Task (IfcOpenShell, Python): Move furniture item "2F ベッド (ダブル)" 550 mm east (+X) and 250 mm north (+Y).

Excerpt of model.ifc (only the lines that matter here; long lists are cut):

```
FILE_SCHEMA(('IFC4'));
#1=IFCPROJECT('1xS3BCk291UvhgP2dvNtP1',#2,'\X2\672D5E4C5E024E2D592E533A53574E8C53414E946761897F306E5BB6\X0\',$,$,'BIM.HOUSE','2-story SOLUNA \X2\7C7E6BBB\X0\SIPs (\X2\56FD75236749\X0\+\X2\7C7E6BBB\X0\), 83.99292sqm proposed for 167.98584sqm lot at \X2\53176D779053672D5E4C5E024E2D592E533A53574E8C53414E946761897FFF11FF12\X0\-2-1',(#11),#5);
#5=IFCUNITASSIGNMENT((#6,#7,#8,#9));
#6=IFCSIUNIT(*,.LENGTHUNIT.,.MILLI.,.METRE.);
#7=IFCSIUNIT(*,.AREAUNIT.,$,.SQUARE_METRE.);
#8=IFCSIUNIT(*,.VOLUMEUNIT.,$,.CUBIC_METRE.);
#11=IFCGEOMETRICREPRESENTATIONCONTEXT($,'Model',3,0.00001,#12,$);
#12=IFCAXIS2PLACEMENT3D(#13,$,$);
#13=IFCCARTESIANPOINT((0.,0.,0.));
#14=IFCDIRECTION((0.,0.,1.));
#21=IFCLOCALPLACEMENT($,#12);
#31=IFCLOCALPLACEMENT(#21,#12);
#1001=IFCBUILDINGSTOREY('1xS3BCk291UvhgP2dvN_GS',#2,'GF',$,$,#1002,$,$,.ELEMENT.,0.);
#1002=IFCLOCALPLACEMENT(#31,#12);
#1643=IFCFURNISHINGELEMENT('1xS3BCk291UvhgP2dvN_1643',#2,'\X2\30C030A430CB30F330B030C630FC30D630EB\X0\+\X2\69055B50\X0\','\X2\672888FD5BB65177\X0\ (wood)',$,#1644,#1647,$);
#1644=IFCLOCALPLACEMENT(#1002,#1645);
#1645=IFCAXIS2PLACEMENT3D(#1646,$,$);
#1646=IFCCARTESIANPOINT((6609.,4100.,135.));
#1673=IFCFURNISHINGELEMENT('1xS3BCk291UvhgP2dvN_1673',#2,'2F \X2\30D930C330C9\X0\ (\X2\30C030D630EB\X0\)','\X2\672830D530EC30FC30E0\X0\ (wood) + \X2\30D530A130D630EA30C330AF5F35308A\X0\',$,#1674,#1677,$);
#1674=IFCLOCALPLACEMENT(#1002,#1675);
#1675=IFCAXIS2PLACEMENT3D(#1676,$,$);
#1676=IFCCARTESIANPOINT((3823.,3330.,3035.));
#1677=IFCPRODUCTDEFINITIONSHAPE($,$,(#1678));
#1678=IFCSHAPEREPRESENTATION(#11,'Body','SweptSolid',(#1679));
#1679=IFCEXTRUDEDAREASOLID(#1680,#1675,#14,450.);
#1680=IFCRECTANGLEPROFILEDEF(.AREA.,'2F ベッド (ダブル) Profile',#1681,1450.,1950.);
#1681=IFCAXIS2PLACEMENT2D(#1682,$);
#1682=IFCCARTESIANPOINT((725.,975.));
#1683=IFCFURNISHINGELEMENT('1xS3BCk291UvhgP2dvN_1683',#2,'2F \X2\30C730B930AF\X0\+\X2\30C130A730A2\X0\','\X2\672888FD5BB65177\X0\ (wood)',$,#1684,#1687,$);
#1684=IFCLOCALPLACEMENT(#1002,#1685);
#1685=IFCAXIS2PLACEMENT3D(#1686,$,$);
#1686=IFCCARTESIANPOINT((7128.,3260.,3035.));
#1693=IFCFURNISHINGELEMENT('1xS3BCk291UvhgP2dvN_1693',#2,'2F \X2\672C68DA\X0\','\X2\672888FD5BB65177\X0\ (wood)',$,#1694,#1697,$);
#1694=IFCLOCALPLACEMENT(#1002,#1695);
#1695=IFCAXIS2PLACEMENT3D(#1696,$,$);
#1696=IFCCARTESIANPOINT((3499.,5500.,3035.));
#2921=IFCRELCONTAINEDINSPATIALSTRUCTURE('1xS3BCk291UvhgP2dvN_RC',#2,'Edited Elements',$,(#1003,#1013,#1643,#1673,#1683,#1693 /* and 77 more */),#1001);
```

```python
import ifcopenshell
import ifcopenshell.api.geometry
import ifcopenshell.util.placement
import ifcopenshell.util.unit

model = ifcopenshell.open("model.ifc")
unit_scale = ifcopenshell.util.unit.calculate_unit_scale(model)

item = model.by_guid("1xS3BCk291UvhgP2dvN_1673")
matrix = ifcopenshell.util.placement.get_local_placement(item.ObjectPlacement)
matrix[0, 3] += 0.55 / unit_scale
matrix[1, 3] += 0.25 / unit_scale
ifcopenshell.api.geometry.edit_object_placement(model, product=item, matrix=matrix, is_si=False)

print(ifcopenshell.util.placement.get_local_placement(item.ObjectPlacement).round(3) + 0.0)

model.write("model_updated.ifc")
```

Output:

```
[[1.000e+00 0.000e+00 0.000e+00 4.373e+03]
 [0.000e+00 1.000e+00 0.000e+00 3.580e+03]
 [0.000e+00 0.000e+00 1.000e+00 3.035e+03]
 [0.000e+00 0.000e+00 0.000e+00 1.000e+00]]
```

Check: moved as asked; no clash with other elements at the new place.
